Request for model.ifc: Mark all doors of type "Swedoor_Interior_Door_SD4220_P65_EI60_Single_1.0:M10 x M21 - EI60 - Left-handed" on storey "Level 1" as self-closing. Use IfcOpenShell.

First a look at what the model holds.

```python
import ifcopenshell
import ifcopenshell.util.element

model = ifcopenshell.open("model.ifc")
print(model.schema)
storey = next(s for s in model.by_type("IfcBuildingStorey") if s.Name == "Level 1")
doors = [e for e in ifcopenshell.util.element.get_decomposition(storey) if e.is_a("IfcDoor")]
seen = {}
for e in doors:
    element_type = ifcopenshell.util.element.get_type(e)
    key = (element_type.Name if element_type != e and element_type else None, ifcopenshell.util.element.get_pset(e, "Pset_DoorCommon", "SelfClosing"))
    seen[key] = seen.get(key, 0) + 1
for (name, value), count in sorted(seen.items(), key=str):
    print(count, "x", name, "|", value)
```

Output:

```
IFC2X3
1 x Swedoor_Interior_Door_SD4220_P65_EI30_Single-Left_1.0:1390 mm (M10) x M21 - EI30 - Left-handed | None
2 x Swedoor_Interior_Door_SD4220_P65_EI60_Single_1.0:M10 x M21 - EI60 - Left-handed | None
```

```python
import ifcopenshell
import ifcopenshell.api.pset
import ifcopenshell.util.element

model = ifcopenshell.open("model.ifc")

storey = next(s for s in model.by_type("IfcBuildingStorey") if s.Name == "Level 1")
doors = [e for e in ifcopenshell.util.element.get_decomposition(storey) if e.is_a("IfcDoor")]

count = 0
for e in doors:
    element_type = ifcopenshell.util.element.get_type(e)
    if element_type in (None, e) or element_type.Name != "Swedoor_Interior_Door_SD4220_P65_EI60_Single_1.0:M10 x M21 - EI60 - Left-handed":
        continue
    # add_pset returns the element's existing set when there is one.
    pset = ifcopenshell.api.pset.add_pset(model, product=e, name="Pset_DoorCommon")
    ifcopenshell.api.pset.edit_pset(model, pset=pset, properties={"SelfClosing": True})
    count += 1

print(count, "doors updated")

model.write("model_v2.ifc")
```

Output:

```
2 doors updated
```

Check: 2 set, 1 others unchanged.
